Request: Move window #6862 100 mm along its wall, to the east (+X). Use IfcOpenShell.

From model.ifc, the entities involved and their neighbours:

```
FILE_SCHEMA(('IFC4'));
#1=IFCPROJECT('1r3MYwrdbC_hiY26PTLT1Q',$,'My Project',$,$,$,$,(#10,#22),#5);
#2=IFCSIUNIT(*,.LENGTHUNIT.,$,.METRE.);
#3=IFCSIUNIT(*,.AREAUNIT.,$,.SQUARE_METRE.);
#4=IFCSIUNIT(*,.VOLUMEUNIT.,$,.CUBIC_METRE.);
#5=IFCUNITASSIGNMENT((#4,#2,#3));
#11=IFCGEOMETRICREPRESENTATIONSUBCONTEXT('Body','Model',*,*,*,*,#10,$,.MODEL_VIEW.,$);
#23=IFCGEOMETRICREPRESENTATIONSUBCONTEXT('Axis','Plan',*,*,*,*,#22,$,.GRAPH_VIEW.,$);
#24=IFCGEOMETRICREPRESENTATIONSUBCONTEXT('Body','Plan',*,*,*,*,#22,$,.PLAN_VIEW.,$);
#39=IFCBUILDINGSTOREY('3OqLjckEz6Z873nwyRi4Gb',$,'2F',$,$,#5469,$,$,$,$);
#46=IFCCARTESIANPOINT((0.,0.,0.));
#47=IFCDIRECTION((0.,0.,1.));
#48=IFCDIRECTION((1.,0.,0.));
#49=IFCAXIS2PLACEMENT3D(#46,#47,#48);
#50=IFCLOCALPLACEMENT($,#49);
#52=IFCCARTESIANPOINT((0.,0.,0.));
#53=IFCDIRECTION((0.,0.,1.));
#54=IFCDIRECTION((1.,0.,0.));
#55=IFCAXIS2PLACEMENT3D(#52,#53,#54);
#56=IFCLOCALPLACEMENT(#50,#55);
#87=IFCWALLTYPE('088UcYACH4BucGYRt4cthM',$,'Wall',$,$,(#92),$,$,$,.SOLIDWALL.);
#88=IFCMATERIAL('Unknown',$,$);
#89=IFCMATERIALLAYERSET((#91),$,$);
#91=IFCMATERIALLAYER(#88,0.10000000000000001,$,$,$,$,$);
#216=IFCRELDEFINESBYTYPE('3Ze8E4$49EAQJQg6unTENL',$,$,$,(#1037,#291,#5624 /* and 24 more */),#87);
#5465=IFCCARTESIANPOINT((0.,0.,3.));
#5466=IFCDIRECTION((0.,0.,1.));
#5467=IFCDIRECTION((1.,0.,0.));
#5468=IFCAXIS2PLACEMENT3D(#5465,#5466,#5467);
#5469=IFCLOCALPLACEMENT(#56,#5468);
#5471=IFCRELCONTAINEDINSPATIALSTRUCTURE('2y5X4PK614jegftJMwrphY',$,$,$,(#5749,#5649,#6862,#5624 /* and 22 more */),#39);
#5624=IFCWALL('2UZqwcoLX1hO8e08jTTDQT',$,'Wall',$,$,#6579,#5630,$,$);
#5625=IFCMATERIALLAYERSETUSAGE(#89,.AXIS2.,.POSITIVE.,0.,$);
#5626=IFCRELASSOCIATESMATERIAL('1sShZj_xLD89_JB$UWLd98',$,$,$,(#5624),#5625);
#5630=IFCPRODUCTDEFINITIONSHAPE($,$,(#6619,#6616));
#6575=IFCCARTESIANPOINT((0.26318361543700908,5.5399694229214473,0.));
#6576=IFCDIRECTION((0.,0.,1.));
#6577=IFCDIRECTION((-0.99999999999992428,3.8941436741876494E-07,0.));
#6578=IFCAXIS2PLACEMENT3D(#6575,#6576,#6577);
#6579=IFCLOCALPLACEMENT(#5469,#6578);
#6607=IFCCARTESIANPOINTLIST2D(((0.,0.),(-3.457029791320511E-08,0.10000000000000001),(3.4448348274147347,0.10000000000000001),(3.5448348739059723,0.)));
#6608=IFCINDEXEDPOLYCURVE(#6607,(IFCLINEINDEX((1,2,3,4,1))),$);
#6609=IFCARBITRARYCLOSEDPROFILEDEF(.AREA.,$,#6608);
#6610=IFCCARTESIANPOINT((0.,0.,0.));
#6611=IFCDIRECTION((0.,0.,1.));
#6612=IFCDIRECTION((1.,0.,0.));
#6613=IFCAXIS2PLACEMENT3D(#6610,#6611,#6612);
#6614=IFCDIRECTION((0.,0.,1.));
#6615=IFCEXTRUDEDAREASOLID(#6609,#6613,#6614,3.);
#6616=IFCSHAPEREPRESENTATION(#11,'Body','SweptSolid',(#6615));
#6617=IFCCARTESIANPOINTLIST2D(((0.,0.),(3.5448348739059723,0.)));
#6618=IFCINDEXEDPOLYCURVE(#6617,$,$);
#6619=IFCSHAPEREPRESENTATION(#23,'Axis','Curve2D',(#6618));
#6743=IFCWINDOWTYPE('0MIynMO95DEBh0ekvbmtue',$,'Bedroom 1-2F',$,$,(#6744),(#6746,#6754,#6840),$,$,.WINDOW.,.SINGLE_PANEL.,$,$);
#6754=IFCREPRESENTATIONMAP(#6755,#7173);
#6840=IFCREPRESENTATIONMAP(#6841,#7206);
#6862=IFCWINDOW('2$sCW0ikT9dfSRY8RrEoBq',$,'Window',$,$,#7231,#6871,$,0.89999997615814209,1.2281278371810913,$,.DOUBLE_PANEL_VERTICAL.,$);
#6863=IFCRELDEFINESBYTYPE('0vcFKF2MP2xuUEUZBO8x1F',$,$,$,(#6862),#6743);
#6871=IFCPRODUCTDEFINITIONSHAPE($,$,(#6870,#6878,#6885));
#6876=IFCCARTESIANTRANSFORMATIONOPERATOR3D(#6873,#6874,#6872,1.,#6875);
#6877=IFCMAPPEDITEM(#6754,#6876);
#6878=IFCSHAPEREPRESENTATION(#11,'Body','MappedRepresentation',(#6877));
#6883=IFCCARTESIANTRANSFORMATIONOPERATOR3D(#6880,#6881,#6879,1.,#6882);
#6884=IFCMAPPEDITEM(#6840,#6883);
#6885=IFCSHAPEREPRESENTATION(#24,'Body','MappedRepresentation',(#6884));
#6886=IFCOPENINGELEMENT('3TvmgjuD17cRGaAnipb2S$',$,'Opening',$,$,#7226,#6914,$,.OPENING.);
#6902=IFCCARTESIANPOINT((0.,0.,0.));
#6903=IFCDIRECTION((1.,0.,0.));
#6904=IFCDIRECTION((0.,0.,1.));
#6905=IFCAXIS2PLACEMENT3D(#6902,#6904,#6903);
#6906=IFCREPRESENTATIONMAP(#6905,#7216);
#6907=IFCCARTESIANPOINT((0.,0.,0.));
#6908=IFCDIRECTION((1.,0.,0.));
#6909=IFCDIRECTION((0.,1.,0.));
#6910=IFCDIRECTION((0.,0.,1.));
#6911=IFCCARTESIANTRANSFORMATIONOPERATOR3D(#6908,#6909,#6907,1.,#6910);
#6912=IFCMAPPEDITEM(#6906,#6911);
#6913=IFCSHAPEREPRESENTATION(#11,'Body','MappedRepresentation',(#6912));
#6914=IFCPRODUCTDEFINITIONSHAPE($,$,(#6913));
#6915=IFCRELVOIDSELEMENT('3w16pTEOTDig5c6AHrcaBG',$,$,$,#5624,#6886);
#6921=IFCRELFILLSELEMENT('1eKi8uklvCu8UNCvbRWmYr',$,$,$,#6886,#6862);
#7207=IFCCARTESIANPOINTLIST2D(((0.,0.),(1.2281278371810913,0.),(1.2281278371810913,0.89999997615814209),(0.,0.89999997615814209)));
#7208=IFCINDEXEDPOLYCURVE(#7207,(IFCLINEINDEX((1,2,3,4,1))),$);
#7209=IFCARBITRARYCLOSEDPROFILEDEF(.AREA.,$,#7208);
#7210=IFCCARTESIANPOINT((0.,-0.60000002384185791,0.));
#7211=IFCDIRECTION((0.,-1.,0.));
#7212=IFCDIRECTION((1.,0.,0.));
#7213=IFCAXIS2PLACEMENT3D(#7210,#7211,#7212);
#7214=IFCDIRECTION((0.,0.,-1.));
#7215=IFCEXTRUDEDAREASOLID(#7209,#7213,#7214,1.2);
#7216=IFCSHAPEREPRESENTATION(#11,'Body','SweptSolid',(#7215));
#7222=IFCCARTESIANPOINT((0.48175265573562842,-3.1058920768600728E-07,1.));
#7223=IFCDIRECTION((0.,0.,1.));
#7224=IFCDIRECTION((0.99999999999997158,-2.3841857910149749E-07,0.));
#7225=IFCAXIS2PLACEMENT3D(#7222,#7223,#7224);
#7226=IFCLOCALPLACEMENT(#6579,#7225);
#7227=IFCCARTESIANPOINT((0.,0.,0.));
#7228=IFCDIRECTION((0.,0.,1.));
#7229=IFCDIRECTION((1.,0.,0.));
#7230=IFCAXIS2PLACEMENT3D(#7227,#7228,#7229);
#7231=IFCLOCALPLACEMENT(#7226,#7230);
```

```python
import ifcopenshell
import ifcopenshell.api.geometry
import ifcopenshell.util.placement

model = ifcopenshell.open("model.ifc")

window = model.by_guid("2$sCW0ikT9dfSRY8RrEoBq")
opening = window.FillsVoids[0].RelatingOpeningElement
wall = opening.VoidsElements[0].RelatingBuildingElement

wall_matrix = ifcopenshell.util.placement.get_local_placement(wall.ObjectPlacement)
shift = wall_matrix[:3, 0] * -0.1
before = ifcopenshell.util.placement.get_local_placement(window.ObjectPlacement)[:3, 3].copy()

# The window is placed relative to its opening, so it follows when the opening moves.
matrix = ifcopenshell.util.placement.get_local_placement(opening.ObjectPlacement)
matrix[:3, 3] += shift
ifcopenshell.api.geometry.edit_object_placement(
    model, product=opening, matrix=matrix, is_si=False, should_transform_children=True
)

after = ifcopenshell.util.placement.get_local_placement(window.ObjectPlacement)[:3, 3]
print("window moved by", (after - before).round(3) + 0.0)

model.write("model_v2.ifc")
```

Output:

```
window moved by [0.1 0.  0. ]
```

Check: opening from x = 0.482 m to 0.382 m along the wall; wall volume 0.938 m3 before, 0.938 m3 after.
